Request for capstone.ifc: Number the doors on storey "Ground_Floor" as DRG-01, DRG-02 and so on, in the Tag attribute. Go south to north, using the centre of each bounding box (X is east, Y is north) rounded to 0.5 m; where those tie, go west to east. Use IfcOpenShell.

First a look at what the model holds.

```python
import ifcopenshell
import ifcopenshell.util.element
import ifcopenshell.util.placement

model = ifcopenshell.open("capstone.ifc")
print(model.schema)
storey = next(s for s in model.by_type("IfcBuildingStorey") if s.Name == "Ground_Floor")
doors = [e for e in ifcopenshell.util.element.get_decomposition(storey) if e.is_a("IfcDoor")]
for e in sorted(doors, key=lambda e: e.id()):
    origin = ifcopenshell.util.placement.get_local_placement(e.ObjectPlacement)[:3, 3]
    print(e.id(), e.Tag, e.Name, origin.round(2) + 0.0, sep=" | ")
```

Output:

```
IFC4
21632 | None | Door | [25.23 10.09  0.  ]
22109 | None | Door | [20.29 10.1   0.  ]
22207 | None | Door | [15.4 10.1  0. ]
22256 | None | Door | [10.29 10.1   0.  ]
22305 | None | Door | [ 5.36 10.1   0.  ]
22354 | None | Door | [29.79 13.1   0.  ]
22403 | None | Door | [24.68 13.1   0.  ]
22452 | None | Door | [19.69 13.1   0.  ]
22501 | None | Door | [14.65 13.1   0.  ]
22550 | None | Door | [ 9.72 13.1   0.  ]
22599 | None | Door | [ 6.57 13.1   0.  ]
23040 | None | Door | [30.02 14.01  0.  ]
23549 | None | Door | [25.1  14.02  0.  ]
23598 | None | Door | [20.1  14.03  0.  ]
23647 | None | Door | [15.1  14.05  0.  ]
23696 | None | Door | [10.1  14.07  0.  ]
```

```python
import ifcopenshell
import ifcopenshell.geom
import ifcopenshell.util.element
import ifcopenshell.util.shape

model = ifcopenshell.open("capstone.ifc")
settings = ifcopenshell.geom.settings()
settings.set("use-world-coords", True)


def centre(element):
    shape = ifcopenshell.geom.create_shape(settings, element)
    return ifcopenshell.util.shape.get_bbox_centroid(shape.geometry)


storey = next(s for s in model.by_type("IfcBuildingStorey") if s.Name == "Ground_Floor")
doors = [e for e in ifcopenshell.util.element.get_decomposition(storey) if e.is_a("IfcDoor")]

# Insertion points can sit at a corner or the storey origin, so sort by the geometry (in metres).
centres = {e: centre(e) for e in doors}
doors.sort(key=lambda e: (round(centres[e][1] / 0.5), centres[e][0]))

for i, e in enumerate(doors, start=1):
    number = f"DRG-{i:02d}"
    e.Tag = number
    print(e.id(), number)

model.write("capstone_updated.ifc")
```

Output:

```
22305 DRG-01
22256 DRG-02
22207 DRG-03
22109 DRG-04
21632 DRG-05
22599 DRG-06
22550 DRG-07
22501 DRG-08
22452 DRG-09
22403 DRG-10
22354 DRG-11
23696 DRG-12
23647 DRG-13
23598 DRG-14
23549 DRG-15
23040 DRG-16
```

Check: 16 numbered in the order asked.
